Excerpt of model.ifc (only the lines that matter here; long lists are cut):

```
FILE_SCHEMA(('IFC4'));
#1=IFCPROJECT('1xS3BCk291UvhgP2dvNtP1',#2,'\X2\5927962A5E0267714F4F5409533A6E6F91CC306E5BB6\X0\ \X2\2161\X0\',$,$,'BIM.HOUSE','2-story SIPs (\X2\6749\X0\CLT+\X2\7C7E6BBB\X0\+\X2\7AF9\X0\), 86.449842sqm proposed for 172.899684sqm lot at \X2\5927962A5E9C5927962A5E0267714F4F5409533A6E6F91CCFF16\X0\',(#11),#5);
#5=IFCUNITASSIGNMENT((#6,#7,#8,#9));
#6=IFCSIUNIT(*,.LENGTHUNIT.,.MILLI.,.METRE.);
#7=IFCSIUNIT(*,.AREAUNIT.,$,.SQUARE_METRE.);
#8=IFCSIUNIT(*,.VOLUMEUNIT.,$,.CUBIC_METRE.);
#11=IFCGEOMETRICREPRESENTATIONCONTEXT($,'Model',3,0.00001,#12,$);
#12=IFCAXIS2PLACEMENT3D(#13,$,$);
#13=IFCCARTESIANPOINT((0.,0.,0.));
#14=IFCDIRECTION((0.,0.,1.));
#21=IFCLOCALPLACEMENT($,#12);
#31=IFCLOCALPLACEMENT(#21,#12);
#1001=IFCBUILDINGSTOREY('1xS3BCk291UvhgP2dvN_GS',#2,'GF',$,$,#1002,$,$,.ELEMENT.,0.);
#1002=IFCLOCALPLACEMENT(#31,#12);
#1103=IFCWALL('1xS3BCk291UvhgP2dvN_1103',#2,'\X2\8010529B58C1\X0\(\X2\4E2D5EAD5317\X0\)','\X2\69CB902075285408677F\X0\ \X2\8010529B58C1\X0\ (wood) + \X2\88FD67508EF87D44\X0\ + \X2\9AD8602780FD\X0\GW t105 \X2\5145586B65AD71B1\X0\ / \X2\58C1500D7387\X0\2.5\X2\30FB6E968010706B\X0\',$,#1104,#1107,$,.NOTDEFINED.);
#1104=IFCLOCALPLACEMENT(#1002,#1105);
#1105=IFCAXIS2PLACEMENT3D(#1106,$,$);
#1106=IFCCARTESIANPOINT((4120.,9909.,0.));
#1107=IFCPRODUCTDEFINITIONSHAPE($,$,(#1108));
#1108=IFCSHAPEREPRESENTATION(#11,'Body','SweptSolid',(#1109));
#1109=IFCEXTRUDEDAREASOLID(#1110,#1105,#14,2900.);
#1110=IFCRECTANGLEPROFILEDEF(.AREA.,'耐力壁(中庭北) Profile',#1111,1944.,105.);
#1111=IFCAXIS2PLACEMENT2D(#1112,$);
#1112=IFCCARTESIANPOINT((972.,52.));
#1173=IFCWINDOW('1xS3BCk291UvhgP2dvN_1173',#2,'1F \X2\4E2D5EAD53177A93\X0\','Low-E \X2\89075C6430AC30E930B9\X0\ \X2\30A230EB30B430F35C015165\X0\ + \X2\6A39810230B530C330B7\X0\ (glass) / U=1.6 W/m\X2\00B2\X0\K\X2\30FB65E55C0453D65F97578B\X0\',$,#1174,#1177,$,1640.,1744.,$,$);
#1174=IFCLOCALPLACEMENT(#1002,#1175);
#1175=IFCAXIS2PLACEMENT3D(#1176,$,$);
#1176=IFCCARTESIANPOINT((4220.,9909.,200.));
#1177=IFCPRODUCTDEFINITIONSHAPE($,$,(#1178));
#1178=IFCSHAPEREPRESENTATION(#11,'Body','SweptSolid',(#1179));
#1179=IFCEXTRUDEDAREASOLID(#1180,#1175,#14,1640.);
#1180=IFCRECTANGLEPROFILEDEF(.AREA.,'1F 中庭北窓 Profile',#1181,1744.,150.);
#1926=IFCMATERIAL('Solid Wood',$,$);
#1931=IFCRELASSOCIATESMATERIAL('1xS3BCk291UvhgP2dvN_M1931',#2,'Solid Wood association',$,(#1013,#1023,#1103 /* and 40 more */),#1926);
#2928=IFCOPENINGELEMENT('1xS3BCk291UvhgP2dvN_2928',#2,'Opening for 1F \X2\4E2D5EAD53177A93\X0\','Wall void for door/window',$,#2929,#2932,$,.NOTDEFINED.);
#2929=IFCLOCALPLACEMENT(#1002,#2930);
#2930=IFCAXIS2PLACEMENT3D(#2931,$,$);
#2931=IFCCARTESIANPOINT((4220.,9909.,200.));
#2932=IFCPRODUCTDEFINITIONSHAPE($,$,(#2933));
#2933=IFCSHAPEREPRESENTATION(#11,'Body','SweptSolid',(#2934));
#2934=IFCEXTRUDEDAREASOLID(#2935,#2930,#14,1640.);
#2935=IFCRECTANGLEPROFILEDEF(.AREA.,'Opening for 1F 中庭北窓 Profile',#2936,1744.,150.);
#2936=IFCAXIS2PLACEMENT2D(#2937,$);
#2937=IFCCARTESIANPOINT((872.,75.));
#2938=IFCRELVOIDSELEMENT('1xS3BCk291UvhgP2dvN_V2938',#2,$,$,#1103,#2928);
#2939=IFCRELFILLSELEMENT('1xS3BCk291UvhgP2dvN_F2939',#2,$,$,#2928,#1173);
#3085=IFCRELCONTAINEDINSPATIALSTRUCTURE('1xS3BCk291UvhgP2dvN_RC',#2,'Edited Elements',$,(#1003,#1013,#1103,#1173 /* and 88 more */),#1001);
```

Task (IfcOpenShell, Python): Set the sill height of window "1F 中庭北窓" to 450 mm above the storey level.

```python
import numpy as np
import ifcopenshell
import ifcopenshell.api.geometry
import ifcopenshell.geom
import ifcopenshell.util.element
import ifcopenshell.util.placement
import ifcopenshell.util.shape
import ifcopenshell.util.unit

model = ifcopenshell.open("model.ifc")
unit_scale = ifcopenshell.util.unit.calculate_unit_scale(model)

window = model.by_guid("1xS3BCk291UvhgP2dvN_1173")
opening = window.FillsVoids[0].RelatingOpeningElement
storey = ifcopenshell.util.element.get_container(window, ifc_class="IfcBuildingStorey")
level = ifcopenshell.util.placement.get_local_placement(storey.ObjectPlacement)[2, 3]

# The opening's origin need not be at the sill, so measure its lowest point.
shape = ifcopenshell.geom.create_shape(ifcopenshell.geom.settings(), opening)
bottom = ifcopenshell.util.shape.get_shape_bottom_elevation(shape, shape.geometry) / unit_scale
dz = level + 0.45 / unit_scale - bottom

shift = np.array([0.0, 0.0, dz])
# The window is not placed relative to its opening, so move both.
for product in (opening, window):
    matrix = ifcopenshell.util.placement.get_local_placement(product.ObjectPlacement)
    matrix[:3, 3] += shift
    ifcopenshell.api.geometry.edit_object_placement(model, product=product, matrix=matrix, is_si=False)

print(f"moved by {dz * unit_scale:+.3f} m")

model.write("model-out.ifc")
```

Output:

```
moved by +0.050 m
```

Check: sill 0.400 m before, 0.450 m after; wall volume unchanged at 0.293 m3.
